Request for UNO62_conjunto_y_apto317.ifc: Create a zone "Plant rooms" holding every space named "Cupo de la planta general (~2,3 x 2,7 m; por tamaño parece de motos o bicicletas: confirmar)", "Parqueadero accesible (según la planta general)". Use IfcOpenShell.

First a look at what the model holds.

```python
import ifcopenshell

model = ifcopenshell.open("UNO62_conjunto_y_apto317.ifc")
print(model.schema)
seen = {}
for space in model.by_type("IfcSpace"):
    seen[space.LongName] = seen.get(space.LongName, 0) + 1
for name, count in sorted(seen.items(), key=str):
    print(count, "x", name)
print("zones:", [z.Name for z in model.by_type("IfcZone")][:20])
```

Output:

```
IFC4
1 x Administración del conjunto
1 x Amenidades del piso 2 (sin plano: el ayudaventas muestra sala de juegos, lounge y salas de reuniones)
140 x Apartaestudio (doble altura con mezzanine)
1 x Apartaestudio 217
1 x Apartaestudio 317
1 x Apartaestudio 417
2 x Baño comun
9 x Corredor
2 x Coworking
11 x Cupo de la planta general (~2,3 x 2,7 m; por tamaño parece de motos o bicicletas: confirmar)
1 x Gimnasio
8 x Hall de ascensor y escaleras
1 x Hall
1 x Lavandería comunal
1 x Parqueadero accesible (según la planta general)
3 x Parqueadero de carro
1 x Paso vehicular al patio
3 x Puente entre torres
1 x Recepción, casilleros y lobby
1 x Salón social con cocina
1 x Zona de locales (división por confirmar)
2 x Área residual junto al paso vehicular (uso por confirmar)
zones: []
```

```python
import ifcopenshell
import ifcopenshell.api.group
import ifcopenshell.api.root

model = ifcopenshell.open("UNO62_conjunto_y_apto317.ifc")

names = {"Cupo de la planta general (~2,3 x 2,7 m; por tamaño parece de motos o bicicletas: confirmar)", "Parqueadero accesible (según la planta general)"}
spaces = [s for s in model.by_type("IfcSpace") if s.LongName in names]

zone = ifcopenshell.api.root.create_entity(model, ifc_class="IfcZone", name="Plant rooms")
ifcopenshell.api.group.assign_group(model, products=spaces, group=zone)
print(len(spaces), "spaces in", zone.Name)

model.write("UNO62_conjunto_y_apto317-out.ifc")
```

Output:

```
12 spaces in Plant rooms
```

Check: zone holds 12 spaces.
